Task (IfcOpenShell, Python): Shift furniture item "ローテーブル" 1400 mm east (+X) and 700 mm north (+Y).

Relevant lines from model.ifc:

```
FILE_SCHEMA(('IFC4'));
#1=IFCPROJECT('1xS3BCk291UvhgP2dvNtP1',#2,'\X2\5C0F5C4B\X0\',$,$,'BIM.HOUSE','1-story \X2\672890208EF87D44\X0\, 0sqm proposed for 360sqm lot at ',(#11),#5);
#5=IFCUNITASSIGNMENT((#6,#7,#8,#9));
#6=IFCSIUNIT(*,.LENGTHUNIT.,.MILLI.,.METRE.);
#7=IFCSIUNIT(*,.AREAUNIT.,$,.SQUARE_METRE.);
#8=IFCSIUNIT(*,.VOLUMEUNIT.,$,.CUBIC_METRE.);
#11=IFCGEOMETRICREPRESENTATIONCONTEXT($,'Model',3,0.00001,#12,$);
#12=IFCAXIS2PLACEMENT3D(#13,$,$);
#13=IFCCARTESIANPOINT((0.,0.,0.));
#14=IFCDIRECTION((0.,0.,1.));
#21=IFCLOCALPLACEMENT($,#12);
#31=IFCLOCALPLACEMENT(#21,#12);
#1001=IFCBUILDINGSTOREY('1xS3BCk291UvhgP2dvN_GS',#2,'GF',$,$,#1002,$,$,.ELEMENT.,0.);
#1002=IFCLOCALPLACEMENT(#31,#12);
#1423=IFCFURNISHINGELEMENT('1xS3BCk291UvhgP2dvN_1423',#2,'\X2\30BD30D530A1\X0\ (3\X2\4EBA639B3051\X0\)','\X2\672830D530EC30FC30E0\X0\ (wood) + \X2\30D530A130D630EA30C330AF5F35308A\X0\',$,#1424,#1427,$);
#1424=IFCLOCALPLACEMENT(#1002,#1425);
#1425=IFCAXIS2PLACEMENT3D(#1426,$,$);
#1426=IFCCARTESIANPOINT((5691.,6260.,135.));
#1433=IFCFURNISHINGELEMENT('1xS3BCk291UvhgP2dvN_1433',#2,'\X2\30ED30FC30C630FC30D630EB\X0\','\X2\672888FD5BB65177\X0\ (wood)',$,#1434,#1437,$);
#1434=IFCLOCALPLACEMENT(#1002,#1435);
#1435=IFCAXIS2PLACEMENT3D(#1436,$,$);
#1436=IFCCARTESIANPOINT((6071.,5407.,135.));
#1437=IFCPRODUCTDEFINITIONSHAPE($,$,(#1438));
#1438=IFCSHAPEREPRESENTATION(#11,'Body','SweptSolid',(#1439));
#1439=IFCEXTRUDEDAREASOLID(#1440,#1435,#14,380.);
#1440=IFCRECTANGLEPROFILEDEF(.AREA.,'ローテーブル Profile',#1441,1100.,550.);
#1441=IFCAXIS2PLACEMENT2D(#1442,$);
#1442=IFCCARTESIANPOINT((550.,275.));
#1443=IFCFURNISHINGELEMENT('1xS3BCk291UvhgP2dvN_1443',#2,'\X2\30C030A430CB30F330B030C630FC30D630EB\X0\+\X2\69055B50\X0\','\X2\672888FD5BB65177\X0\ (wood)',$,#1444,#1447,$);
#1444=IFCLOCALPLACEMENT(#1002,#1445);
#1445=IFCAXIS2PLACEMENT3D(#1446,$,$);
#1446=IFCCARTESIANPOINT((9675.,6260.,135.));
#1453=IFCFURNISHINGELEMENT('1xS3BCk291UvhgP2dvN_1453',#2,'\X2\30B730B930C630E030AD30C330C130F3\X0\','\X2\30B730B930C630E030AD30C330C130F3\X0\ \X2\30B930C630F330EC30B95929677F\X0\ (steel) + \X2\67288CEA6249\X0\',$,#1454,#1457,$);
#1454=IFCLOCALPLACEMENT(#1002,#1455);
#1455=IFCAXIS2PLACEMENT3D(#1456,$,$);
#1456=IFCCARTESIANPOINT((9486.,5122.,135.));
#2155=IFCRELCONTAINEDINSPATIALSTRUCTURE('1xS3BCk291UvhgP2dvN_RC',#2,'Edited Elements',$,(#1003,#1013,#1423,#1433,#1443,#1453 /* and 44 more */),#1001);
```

```python
import ifcopenshell
import ifcopenshell.api.geometry
import ifcopenshell.util.placement
import ifcopenshell.util.unit

model = ifcopenshell.open("model.ifc")
unit_scale = ifcopenshell.util.unit.calculate_unit_scale(model)

item = model.by_guid("1xS3BCk291UvhgP2dvN_1433")
matrix = ifcopenshell.util.placement.get_local_placement(item.ObjectPlacement)
matrix[0, 3] += 1.4 / unit_scale
matrix[1, 3] += 0.7 / unit_scale
ifcopenshell.api.geometry.edit_object_placement(model, product=item, matrix=matrix, is_si=False)

print(ifcopenshell.util.placement.get_local_placement(item.ObjectPlacement).round(3) + 0.0)

model.write("model_updated.ifc")
```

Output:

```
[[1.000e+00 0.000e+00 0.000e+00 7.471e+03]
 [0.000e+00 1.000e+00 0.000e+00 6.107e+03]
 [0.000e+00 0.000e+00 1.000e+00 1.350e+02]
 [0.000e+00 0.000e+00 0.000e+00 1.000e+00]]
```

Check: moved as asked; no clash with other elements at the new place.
